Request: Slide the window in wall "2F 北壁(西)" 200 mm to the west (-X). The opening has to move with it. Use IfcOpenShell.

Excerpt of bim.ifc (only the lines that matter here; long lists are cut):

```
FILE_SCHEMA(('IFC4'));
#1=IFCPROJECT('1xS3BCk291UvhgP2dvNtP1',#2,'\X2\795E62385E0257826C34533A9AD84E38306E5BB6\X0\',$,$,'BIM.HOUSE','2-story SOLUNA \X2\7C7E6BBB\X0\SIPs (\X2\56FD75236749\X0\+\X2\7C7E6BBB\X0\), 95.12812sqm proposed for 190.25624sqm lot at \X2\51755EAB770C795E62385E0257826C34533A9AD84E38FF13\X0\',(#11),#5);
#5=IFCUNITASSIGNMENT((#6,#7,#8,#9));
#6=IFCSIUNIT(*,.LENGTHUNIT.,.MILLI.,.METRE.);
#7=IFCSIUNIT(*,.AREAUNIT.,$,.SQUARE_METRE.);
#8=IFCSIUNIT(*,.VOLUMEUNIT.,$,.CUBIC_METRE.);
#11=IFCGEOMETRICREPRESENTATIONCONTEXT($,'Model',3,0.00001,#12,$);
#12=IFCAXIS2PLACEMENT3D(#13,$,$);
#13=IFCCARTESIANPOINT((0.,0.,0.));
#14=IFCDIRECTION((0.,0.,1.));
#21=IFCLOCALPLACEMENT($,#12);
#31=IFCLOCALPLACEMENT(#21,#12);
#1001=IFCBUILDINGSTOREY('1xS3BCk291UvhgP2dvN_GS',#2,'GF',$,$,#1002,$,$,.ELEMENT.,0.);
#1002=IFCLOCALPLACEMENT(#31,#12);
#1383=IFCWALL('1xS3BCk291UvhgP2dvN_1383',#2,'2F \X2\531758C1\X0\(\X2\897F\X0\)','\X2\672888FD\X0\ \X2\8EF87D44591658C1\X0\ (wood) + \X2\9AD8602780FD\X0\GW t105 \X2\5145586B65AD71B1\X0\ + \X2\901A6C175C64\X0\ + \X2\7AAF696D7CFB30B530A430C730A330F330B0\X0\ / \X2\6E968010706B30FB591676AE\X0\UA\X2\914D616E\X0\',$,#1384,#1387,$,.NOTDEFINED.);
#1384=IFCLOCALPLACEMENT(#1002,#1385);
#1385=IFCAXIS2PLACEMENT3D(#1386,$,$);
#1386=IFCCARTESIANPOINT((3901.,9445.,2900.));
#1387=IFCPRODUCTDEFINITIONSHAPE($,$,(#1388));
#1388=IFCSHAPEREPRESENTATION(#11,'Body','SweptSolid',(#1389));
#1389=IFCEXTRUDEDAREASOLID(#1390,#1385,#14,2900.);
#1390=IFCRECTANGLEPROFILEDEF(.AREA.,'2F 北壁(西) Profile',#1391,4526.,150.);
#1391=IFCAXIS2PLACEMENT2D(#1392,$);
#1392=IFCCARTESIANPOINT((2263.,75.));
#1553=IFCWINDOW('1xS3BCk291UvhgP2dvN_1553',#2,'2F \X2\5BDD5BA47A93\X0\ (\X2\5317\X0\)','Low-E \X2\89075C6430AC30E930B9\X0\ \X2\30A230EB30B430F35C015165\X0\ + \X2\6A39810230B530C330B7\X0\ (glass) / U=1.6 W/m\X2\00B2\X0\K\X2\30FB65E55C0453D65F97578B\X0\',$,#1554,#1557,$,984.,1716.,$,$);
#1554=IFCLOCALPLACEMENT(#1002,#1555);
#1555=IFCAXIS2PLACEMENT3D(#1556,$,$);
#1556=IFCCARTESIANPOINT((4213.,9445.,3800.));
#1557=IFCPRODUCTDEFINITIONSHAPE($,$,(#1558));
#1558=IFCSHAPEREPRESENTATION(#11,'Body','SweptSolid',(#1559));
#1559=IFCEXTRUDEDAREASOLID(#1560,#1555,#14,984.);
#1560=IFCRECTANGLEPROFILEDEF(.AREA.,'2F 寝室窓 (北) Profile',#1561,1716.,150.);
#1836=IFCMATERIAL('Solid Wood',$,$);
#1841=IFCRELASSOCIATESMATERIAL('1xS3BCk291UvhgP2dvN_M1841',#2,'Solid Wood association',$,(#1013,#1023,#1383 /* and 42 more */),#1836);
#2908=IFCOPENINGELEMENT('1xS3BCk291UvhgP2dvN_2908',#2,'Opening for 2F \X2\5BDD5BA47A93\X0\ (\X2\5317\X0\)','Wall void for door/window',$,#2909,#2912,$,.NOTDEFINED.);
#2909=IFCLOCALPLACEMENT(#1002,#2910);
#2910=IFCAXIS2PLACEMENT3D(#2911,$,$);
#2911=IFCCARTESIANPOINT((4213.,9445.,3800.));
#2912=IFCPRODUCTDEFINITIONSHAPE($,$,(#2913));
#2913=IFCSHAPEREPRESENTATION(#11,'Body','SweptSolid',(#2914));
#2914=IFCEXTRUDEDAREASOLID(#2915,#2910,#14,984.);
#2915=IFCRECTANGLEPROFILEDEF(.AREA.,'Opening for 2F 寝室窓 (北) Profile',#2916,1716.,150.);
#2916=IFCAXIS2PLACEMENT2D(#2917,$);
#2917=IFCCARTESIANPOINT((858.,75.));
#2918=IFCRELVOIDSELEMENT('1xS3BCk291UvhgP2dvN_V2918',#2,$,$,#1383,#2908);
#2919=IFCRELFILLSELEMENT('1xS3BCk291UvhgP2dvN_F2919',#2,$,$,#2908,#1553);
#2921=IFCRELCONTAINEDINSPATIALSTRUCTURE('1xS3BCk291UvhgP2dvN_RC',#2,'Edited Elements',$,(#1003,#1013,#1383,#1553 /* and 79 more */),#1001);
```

```python
import ifcopenshell
import ifcopenshell.api.geometry
import ifcopenshell.util.placement

model = ifcopenshell.open("bim.ifc")

window = model.by_id(1553)
opening = window.FillsVoids[0].RelatingOpeningElement
wall = opening.VoidsElements[0].RelatingBuildingElement

wall_matrix = ifcopenshell.util.placement.get_local_placement(wall.ObjectPlacement)
shift = wall_matrix[:3, 0] * -200.0
before = ifcopenshell.util.placement.get_local_placement(window.ObjectPlacement)[:3, 3].copy()

# The window is not placed relative to its opening, so move both.
for product in (opening, window):
    matrix = ifcopenshell.util.placement.get_local_placement(product.ObjectPlacement)
    matrix[:3, 3] += shift
    ifcopenshell.api.geometry.edit_object_placement(model, product=product, matrix=matrix, is_si=False)

after = ifcopenshell.util.placement.get_local_placement(window.ObjectPlacement)[:3, 3]
print("window moved by", (after - before).round(3) + 0.0)

model.write("bim-out.ifc")
```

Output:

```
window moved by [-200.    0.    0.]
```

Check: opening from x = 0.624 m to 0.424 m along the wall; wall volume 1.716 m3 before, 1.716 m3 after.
